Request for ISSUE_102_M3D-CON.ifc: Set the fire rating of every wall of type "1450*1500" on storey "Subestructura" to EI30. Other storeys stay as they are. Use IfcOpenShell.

First a look at what the model holds.

```python
import ifcopenshell
import ifcopenshell.util.element

model = ifcopenshell.open("ISSUE_102_M3D-CON.ifc")
print(model.schema)
storey = next(s for s in model.by_type("IfcBuildingStorey") if s.Name == "Subestructura")
walls = [e for e in ifcopenshell.util.element.get_decomposition(storey) if e.is_a("IfcWall")]
seen = {}
for e in walls:
    element_type = ifcopenshell.util.element.get_type(e)
    key = (element_type.Name if element_type != e and element_type else None, ifcopenshell.util.element.get_pset(e, "Pset_WallCommon", "FireRating"))
    seen[key] = seen.get(key, 0) + 1
for (name, value), count in sorted(seen.items(), key=str):
    print(count, "x", name, "|", value)
```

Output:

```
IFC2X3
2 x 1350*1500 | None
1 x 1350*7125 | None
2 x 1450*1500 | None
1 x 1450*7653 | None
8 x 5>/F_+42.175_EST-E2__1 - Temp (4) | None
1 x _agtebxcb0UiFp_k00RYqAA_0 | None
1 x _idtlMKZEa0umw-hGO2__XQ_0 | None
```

```python
import ifcopenshell
import ifcopenshell.api.pset
import ifcopenshell.util.element

model = ifcopenshell.open("ISSUE_102_M3D-CON.ifc")

storey = next(s for s in model.by_type("IfcBuildingStorey") if s.Name == "Subestructura")
walls = [e for e in ifcopenshell.util.element.get_decomposition(storey) if e.is_a("IfcWall")]

count = 0
for e in walls:
    element_type = ifcopenshell.util.element.get_type(e)
    if element_type in (None, e) or element_type.Name != "1450*1500":
        continue
    found = ifcopenshell.util.element.get_pset(e, "Pset_WallCommon", should_inherit=False)
    if found:
        pset = model.by_id(found["id"])
        if len(ifcopenshell.util.element.get_elements_by_pset(pset)) > 1:
            pset = ifcopenshell.api.pset.unshare_pset(model, products=[e], pset=pset)[0]
    else:
        pset = ifcopenshell.api.pset.add_pset(model, product=e, name="Pset_WallCommon")
    ifcopenshell.api.pset.edit_pset(model, pset=pset, properties={"FireRating": "EI30"})
    count += 1

print(count, "walls updated")

model.write("ISSUE_102_M3D-CON-out.ifc")
```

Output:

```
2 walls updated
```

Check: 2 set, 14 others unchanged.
